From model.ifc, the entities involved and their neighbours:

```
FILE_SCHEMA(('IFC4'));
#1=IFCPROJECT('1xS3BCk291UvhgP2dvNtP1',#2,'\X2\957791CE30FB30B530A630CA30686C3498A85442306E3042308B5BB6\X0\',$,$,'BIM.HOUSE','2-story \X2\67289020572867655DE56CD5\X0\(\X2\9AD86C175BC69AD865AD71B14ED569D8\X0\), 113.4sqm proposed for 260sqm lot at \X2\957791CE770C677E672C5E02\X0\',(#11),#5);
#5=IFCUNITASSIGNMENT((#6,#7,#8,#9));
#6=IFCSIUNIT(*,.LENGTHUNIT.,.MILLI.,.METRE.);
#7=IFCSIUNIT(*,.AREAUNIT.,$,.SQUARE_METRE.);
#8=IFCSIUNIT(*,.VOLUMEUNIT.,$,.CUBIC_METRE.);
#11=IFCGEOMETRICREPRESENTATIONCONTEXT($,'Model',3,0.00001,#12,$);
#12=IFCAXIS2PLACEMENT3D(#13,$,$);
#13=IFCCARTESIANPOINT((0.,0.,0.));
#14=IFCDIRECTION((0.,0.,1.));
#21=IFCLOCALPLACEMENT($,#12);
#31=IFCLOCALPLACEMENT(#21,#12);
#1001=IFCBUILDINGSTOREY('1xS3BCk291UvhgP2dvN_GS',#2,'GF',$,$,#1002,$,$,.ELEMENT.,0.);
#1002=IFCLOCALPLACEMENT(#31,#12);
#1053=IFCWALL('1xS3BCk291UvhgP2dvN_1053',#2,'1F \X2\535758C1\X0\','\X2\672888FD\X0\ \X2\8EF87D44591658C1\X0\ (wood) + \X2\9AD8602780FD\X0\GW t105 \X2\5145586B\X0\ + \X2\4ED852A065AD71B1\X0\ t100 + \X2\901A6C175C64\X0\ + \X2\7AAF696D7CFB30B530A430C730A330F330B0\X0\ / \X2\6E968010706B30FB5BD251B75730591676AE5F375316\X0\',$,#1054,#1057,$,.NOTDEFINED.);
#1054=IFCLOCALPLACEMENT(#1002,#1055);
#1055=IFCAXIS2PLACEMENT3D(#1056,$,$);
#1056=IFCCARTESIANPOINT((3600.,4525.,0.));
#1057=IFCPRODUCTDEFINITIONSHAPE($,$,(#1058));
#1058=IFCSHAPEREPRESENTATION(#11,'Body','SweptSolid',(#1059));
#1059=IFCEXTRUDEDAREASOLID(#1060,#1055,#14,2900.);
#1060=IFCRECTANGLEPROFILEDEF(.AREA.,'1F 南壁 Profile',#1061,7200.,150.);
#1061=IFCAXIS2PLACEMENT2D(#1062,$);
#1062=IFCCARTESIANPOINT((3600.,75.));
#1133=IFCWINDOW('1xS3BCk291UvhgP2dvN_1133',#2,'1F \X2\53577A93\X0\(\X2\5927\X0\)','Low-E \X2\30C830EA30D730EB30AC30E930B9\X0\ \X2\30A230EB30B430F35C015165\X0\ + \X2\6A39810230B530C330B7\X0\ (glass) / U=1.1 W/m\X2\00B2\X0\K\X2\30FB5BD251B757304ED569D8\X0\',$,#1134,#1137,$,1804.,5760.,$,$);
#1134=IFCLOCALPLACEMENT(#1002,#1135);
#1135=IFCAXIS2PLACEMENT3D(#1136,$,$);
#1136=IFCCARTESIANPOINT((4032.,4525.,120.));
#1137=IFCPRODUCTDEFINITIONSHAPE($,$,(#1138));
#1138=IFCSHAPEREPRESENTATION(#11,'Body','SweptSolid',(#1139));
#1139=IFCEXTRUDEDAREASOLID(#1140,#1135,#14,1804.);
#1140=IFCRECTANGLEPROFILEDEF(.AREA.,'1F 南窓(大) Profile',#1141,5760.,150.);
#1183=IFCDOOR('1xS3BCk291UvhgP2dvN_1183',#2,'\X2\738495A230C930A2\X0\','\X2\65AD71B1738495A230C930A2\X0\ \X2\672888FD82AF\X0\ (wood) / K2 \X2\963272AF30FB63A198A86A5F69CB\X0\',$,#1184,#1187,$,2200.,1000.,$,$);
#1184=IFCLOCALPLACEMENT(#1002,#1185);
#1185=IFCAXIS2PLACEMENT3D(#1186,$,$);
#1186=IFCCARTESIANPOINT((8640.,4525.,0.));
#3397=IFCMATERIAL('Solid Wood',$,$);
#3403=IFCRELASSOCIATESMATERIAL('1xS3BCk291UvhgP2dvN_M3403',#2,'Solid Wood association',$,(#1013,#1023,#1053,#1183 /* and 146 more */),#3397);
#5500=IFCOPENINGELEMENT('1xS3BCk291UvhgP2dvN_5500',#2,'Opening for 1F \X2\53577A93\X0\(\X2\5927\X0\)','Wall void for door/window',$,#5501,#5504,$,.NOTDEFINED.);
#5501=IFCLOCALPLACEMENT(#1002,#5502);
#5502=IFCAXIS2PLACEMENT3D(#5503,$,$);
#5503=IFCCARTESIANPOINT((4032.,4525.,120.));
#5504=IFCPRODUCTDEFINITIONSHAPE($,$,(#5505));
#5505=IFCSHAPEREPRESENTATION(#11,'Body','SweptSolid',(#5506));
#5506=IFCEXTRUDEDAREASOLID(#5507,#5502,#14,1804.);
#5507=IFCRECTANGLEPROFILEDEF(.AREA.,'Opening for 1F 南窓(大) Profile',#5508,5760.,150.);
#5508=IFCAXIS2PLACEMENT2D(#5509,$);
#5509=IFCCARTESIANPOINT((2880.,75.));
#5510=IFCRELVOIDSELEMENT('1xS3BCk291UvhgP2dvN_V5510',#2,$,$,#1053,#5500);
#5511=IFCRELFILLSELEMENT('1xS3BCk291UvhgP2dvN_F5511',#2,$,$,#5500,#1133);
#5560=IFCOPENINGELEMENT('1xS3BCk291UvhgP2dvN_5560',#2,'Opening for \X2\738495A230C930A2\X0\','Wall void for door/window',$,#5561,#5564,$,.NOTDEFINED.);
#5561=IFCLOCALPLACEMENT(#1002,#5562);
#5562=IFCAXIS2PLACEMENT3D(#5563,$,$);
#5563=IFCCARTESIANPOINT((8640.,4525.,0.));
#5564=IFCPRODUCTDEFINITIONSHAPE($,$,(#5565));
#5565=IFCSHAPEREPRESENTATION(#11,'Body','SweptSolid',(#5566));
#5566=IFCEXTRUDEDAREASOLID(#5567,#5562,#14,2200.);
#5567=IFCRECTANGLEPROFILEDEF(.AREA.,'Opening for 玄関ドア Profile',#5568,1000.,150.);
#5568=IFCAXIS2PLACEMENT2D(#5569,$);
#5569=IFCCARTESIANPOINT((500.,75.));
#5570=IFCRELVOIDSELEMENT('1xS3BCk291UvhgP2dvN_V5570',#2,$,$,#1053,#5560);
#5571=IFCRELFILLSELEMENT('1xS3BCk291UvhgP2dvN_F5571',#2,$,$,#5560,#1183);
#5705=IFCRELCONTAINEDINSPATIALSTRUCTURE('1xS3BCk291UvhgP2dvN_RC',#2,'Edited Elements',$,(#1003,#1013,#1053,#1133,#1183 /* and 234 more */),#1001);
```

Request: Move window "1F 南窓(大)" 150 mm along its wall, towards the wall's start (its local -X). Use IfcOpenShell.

```python
import ifcopenshell
import ifcopenshell.api.geometry
import ifcopenshell.util.placement

model = ifcopenshell.open("model.ifc")

window = model.by_guid("1xS3BCk291UvhgP2dvN_1133")
opening = window.FillsVoids[0].RelatingOpeningElement
wall = opening.VoidsElements[0].RelatingBuildingElement

wall_matrix = ifcopenshell.util.placement.get_local_placement(wall.ObjectPlacement)
shift = wall_matrix[:3, 0] * -150.0
before = ifcopenshell.util.placement.get_local_placement(window.ObjectPlacement)[:3, 3].copy()

# The window is not placed relative to its opening, so move both.
for product in (opening, window):
    matrix = ifcopenshell.util.placement.get_local_placement(product.ObjectPlacement)
    matrix[:3, 3] += shift
    ifcopenshell.api.geometry.edit_object_placement(model, product=product, matrix=matrix, is_si=False)

after = ifcopenshell.util.placement.get_local_placement(window.ObjectPlacement)[:3, 3]
print("window moved by", (after - before).round(3) + 0.0)

model.write("model_edited.ifc")
```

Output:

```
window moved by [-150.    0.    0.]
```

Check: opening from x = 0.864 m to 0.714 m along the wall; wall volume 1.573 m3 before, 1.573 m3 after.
